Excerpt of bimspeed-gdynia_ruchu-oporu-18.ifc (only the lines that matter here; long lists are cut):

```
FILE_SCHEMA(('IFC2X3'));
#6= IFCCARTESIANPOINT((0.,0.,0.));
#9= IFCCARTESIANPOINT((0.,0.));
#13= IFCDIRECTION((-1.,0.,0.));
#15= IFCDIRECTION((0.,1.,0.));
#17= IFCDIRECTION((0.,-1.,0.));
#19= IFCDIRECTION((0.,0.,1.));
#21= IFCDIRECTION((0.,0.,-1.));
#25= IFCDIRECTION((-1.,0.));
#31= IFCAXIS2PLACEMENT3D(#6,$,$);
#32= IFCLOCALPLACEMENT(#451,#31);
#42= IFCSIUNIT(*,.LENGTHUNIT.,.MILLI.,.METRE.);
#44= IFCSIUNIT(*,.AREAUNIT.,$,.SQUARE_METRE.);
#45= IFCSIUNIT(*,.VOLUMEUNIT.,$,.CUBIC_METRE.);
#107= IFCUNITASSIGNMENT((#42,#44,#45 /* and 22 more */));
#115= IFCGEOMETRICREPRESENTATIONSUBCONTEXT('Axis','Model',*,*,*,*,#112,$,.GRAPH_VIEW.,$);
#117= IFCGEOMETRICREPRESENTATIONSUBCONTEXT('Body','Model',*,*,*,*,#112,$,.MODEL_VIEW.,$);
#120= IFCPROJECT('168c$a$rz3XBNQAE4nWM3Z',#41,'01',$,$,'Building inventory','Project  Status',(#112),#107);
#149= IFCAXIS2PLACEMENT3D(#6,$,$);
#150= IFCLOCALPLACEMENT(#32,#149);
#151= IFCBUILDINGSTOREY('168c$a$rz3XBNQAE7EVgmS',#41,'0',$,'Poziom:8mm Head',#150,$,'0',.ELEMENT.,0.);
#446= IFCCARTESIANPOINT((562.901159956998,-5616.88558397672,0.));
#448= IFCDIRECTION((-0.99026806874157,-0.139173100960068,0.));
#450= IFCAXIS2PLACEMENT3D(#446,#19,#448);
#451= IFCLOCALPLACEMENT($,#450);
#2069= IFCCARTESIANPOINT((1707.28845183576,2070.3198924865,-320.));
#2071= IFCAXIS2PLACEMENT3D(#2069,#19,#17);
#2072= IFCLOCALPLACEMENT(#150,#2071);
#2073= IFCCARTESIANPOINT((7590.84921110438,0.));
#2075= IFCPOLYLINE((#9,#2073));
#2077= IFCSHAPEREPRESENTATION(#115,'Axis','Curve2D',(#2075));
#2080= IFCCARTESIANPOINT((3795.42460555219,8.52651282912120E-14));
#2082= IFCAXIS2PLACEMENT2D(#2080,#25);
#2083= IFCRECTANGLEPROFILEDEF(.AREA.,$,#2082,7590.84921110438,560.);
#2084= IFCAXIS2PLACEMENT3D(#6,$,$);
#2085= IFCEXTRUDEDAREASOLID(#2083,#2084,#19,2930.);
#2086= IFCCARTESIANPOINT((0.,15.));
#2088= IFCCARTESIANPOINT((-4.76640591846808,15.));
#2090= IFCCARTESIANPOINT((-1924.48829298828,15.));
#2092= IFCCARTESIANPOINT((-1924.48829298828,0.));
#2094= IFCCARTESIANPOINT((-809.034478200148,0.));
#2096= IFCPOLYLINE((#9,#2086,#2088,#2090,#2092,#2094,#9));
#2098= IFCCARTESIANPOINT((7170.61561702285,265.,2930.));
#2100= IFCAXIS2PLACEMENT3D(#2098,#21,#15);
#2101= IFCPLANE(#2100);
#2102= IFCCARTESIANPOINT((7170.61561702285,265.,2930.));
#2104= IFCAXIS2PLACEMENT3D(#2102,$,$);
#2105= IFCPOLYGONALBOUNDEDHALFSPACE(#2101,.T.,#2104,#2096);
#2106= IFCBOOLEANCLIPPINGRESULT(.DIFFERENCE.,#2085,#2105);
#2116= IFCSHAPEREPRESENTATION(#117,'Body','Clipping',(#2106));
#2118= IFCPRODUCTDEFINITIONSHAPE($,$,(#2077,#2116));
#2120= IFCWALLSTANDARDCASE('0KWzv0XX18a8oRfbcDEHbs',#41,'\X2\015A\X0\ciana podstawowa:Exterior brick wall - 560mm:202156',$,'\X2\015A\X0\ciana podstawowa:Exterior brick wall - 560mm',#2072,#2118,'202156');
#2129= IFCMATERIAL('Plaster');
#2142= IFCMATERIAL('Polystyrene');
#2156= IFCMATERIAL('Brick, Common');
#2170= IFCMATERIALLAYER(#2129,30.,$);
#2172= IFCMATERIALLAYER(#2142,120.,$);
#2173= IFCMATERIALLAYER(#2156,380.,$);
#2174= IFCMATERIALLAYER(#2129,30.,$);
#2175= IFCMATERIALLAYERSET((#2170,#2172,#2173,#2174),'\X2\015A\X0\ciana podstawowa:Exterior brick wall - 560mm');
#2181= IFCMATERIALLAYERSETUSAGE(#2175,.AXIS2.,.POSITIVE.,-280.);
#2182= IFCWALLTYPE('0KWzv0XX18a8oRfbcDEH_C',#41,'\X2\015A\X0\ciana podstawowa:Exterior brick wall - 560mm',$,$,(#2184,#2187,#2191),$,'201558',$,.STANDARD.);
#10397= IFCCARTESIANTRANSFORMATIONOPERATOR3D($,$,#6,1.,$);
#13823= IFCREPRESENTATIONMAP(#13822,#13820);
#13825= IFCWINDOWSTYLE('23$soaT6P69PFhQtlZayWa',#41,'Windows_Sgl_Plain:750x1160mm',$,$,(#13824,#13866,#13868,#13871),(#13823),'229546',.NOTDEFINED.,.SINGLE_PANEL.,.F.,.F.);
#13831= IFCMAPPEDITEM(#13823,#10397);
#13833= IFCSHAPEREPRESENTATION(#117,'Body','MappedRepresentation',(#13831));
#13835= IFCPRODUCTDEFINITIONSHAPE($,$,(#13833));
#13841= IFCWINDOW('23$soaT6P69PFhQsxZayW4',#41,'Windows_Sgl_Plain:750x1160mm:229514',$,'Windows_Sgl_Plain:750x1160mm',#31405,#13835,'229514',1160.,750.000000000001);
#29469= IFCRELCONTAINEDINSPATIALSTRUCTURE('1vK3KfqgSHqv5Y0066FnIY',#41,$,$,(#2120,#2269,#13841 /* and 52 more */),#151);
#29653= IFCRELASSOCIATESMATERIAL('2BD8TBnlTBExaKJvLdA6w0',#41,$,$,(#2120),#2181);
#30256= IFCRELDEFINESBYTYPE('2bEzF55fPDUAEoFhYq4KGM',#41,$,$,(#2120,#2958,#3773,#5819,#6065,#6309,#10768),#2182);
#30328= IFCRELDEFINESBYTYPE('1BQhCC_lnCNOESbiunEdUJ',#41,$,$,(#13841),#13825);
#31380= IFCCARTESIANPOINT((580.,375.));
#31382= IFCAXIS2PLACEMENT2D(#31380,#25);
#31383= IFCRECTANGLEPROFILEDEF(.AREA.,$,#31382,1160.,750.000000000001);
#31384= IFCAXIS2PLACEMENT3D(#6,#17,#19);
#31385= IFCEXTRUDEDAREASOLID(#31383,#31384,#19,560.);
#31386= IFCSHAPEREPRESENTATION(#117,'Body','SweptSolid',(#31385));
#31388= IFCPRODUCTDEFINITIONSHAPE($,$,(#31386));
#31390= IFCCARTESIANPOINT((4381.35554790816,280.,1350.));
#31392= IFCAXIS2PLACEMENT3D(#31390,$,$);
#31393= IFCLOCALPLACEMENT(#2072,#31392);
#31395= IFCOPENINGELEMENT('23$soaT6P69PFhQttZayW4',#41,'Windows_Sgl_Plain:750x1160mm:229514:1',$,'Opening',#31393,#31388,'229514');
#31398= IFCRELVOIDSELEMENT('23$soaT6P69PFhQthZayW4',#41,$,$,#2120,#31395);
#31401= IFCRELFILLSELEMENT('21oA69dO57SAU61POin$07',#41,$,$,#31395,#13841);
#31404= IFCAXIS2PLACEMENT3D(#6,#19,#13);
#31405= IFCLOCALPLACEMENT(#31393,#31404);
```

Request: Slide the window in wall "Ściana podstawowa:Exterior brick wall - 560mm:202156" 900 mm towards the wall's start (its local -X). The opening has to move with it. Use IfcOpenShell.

```python
import ifcopenshell
import ifcopenshell.api.geometry
import ifcopenshell.util.placement
import ifcopenshell.util.unit

model = ifcopenshell.open("bimspeed-gdynia_ruchu-oporu-18.ifc")
unit_scale = ifcopenshell.util.unit.calculate_unit_scale(model)

window = model.by_id(13841)
opening = window.FillsVoids[0].RelatingOpeningElement
wall = opening.VoidsElements[0].RelatingBuildingElement

wall_matrix = ifcopenshell.util.placement.get_local_placement(wall.ObjectPlacement)
shift = wall_matrix[:3, 0] * -0.9 / unit_scale
before = ifcopenshell.util.placement.get_local_placement(window.ObjectPlacement)[:3, 3].copy()

# The window is placed relative to its opening, so it follows when the opening moves.
matrix = ifcopenshell.util.placement.get_local_placement(opening.ObjectPlacement)
matrix[:3, 3] += shift
ifcopenshell.api.geometry.edit_object_placement(
    model, product=opening, matrix=matrix, is_si=False, should_transform_children=True
)

after = ifcopenshell.util.placement.get_local_placement(window.ObjectPlacement)[:3, 3]
print("window moved by", (after - before).round(3) + 0.0)

model.write("bimspeed-gdynia_ruchu-oporu-18_edited.ifc")
```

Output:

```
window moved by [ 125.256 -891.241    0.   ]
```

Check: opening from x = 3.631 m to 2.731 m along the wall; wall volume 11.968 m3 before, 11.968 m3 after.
